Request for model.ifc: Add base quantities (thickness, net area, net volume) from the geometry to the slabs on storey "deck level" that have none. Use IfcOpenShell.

First a look at what the model holds.

```python
import ifcopenshell
import ifcopenshell.util.element
import ifcopenshell.util.unit

model = ifcopenshell.open("model.ifc")
print(model.schema)
for unit_type in ("LENGTHUNIT", "AREAUNIT", "VOLUMEUNIT"):
    print(unit_type, ifcopenshell.util.unit.calculate_unit_scale(model, unit_type))
storey = next(s for s in model.by_type("IfcBuildingStorey") if s.Name == "deck level")
slabs = [e for e in ifcopenshell.util.element.get_decomposition(storey) if e.is_a("IfcSlab")]
for e in sorted(slabs, key=lambda e: e.id()):
    print(e.id(), e.is_a(), e.Name, list(ifcopenshell.util.element.get_psets(e, qtos_only=True)), sep=" | ")
```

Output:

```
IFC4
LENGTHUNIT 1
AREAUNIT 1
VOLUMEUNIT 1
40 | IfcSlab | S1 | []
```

```python
import ifcopenshell
import ifcopenshell.api.pset
import ifcopenshell.geom
import ifcopenshell.util.element
import ifcopenshell.util.shape
import ifcopenshell.util.unit

model = ifcopenshell.open("model.ifc")
unit_scale = ifcopenshell.util.unit.calculate_unit_scale(model)
area_scale = ifcopenshell.util.unit.calculate_unit_scale(model, "AREAUNIT")
volume_scale = ifcopenshell.util.unit.calculate_unit_scale(model, "VOLUMEUNIT")
settings = ifcopenshell.geom.settings()

storey = next(s for s in model.by_type("IfcBuildingStorey") if s.Name == "deck level")
slabs = [e for e in ifcopenshell.util.element.get_decomposition(storey) if e.is_a("IfcSlab")]

for e in sorted(slabs, key=lambda e: e.id()):
    if ifcopenshell.util.element.get_psets(e, qtos_only=True, should_inherit=False):
        continue
    # Geometry comes back in metres, in the element's own axes.
    shape = ifcopenshell.geom.create_shape(settings, e)
    values = {
        "Width": ifcopenshell.util.shape.get_z(shape.geometry) / unit_scale,
        "NetArea": ifcopenshell.util.shape.get_footprint_area(shape.geometry) / area_scale,
        "NetVolume": ifcopenshell.util.shape.get_volume(shape.geometry) / volume_scale,
    }
    qto = ifcopenshell.api.pset.add_qto(model, product=e, name="Qto_SlabBaseQuantities")
    ifcopenshell.api.pset.edit_qto(model, qto=qto, properties=values)
    print(e.id(), {k: round(v, 3) for k, v in values.items()})

model.write("model_edited.ifc")
```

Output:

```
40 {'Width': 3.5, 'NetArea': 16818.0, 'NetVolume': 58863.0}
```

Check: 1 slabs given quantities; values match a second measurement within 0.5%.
